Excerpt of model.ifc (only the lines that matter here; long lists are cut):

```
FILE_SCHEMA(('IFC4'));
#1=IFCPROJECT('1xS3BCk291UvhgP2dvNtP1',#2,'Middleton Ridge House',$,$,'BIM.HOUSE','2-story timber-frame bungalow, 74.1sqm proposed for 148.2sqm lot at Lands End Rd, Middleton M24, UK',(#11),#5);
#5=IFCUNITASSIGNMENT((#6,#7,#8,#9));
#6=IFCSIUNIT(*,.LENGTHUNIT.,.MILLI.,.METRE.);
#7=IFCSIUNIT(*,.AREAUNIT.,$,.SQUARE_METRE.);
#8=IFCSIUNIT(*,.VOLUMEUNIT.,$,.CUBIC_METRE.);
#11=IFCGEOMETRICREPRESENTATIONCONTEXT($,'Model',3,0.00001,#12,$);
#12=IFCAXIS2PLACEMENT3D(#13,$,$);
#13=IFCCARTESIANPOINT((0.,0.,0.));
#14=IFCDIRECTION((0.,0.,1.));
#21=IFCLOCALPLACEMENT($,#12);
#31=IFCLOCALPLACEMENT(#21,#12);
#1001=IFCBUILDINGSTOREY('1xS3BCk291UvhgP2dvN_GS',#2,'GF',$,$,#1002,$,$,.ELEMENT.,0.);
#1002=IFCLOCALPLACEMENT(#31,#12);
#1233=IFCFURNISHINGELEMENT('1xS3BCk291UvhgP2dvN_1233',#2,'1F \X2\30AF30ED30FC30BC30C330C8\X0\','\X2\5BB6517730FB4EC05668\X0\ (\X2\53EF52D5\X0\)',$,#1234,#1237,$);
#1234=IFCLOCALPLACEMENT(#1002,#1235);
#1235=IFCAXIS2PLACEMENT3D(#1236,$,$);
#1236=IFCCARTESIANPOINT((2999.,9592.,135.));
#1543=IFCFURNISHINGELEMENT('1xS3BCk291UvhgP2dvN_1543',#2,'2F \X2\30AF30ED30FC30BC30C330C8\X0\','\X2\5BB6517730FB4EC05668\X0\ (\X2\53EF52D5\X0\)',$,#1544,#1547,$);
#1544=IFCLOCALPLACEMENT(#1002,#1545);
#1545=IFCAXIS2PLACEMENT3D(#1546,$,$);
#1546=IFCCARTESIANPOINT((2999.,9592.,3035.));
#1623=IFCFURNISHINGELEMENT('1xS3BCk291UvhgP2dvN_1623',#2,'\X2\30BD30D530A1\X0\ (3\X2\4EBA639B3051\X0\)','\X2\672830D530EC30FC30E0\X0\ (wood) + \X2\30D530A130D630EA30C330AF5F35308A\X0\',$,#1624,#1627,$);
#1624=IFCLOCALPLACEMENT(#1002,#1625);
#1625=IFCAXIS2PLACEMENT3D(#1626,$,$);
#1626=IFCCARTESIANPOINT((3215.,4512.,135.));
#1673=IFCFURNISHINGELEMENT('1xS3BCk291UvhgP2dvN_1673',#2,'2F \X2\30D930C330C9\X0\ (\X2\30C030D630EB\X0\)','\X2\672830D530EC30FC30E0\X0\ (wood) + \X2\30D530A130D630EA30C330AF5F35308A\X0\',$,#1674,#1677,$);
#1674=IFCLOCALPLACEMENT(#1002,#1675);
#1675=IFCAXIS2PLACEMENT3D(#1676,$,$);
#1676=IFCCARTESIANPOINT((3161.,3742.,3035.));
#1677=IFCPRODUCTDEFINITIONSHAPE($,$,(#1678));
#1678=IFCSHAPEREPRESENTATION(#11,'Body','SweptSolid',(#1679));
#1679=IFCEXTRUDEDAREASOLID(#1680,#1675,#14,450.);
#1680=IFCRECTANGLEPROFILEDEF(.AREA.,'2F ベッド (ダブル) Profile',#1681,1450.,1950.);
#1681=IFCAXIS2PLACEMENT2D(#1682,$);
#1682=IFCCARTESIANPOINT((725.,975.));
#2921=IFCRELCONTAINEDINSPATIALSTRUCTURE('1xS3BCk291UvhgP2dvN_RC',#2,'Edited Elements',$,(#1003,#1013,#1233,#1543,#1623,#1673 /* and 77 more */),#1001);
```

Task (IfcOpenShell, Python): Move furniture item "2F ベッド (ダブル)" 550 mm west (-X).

```python
import ifcopenshell
import ifcopenshell.api.geometry
import ifcopenshell.util.placement

model = ifcopenshell.open("model.ifc")

item = model.by_guid("1xS3BCk291UvhgP2dvN_1673")
matrix = ifcopenshell.util.placement.get_local_placement(item.ObjectPlacement)
matrix[0, 3] -= 550.0
ifcopenshell.api.geometry.edit_object_placement(model, product=item, matrix=matrix, is_si=False)

print(ifcopenshell.util.placement.get_local_placement(item.ObjectPlacement).round(3) + 0.0)

model.write("model_edited.ifc")
```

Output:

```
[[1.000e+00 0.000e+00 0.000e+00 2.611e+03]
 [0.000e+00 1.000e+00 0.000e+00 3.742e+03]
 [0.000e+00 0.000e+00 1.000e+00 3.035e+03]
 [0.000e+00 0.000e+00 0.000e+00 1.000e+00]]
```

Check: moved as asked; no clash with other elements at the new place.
